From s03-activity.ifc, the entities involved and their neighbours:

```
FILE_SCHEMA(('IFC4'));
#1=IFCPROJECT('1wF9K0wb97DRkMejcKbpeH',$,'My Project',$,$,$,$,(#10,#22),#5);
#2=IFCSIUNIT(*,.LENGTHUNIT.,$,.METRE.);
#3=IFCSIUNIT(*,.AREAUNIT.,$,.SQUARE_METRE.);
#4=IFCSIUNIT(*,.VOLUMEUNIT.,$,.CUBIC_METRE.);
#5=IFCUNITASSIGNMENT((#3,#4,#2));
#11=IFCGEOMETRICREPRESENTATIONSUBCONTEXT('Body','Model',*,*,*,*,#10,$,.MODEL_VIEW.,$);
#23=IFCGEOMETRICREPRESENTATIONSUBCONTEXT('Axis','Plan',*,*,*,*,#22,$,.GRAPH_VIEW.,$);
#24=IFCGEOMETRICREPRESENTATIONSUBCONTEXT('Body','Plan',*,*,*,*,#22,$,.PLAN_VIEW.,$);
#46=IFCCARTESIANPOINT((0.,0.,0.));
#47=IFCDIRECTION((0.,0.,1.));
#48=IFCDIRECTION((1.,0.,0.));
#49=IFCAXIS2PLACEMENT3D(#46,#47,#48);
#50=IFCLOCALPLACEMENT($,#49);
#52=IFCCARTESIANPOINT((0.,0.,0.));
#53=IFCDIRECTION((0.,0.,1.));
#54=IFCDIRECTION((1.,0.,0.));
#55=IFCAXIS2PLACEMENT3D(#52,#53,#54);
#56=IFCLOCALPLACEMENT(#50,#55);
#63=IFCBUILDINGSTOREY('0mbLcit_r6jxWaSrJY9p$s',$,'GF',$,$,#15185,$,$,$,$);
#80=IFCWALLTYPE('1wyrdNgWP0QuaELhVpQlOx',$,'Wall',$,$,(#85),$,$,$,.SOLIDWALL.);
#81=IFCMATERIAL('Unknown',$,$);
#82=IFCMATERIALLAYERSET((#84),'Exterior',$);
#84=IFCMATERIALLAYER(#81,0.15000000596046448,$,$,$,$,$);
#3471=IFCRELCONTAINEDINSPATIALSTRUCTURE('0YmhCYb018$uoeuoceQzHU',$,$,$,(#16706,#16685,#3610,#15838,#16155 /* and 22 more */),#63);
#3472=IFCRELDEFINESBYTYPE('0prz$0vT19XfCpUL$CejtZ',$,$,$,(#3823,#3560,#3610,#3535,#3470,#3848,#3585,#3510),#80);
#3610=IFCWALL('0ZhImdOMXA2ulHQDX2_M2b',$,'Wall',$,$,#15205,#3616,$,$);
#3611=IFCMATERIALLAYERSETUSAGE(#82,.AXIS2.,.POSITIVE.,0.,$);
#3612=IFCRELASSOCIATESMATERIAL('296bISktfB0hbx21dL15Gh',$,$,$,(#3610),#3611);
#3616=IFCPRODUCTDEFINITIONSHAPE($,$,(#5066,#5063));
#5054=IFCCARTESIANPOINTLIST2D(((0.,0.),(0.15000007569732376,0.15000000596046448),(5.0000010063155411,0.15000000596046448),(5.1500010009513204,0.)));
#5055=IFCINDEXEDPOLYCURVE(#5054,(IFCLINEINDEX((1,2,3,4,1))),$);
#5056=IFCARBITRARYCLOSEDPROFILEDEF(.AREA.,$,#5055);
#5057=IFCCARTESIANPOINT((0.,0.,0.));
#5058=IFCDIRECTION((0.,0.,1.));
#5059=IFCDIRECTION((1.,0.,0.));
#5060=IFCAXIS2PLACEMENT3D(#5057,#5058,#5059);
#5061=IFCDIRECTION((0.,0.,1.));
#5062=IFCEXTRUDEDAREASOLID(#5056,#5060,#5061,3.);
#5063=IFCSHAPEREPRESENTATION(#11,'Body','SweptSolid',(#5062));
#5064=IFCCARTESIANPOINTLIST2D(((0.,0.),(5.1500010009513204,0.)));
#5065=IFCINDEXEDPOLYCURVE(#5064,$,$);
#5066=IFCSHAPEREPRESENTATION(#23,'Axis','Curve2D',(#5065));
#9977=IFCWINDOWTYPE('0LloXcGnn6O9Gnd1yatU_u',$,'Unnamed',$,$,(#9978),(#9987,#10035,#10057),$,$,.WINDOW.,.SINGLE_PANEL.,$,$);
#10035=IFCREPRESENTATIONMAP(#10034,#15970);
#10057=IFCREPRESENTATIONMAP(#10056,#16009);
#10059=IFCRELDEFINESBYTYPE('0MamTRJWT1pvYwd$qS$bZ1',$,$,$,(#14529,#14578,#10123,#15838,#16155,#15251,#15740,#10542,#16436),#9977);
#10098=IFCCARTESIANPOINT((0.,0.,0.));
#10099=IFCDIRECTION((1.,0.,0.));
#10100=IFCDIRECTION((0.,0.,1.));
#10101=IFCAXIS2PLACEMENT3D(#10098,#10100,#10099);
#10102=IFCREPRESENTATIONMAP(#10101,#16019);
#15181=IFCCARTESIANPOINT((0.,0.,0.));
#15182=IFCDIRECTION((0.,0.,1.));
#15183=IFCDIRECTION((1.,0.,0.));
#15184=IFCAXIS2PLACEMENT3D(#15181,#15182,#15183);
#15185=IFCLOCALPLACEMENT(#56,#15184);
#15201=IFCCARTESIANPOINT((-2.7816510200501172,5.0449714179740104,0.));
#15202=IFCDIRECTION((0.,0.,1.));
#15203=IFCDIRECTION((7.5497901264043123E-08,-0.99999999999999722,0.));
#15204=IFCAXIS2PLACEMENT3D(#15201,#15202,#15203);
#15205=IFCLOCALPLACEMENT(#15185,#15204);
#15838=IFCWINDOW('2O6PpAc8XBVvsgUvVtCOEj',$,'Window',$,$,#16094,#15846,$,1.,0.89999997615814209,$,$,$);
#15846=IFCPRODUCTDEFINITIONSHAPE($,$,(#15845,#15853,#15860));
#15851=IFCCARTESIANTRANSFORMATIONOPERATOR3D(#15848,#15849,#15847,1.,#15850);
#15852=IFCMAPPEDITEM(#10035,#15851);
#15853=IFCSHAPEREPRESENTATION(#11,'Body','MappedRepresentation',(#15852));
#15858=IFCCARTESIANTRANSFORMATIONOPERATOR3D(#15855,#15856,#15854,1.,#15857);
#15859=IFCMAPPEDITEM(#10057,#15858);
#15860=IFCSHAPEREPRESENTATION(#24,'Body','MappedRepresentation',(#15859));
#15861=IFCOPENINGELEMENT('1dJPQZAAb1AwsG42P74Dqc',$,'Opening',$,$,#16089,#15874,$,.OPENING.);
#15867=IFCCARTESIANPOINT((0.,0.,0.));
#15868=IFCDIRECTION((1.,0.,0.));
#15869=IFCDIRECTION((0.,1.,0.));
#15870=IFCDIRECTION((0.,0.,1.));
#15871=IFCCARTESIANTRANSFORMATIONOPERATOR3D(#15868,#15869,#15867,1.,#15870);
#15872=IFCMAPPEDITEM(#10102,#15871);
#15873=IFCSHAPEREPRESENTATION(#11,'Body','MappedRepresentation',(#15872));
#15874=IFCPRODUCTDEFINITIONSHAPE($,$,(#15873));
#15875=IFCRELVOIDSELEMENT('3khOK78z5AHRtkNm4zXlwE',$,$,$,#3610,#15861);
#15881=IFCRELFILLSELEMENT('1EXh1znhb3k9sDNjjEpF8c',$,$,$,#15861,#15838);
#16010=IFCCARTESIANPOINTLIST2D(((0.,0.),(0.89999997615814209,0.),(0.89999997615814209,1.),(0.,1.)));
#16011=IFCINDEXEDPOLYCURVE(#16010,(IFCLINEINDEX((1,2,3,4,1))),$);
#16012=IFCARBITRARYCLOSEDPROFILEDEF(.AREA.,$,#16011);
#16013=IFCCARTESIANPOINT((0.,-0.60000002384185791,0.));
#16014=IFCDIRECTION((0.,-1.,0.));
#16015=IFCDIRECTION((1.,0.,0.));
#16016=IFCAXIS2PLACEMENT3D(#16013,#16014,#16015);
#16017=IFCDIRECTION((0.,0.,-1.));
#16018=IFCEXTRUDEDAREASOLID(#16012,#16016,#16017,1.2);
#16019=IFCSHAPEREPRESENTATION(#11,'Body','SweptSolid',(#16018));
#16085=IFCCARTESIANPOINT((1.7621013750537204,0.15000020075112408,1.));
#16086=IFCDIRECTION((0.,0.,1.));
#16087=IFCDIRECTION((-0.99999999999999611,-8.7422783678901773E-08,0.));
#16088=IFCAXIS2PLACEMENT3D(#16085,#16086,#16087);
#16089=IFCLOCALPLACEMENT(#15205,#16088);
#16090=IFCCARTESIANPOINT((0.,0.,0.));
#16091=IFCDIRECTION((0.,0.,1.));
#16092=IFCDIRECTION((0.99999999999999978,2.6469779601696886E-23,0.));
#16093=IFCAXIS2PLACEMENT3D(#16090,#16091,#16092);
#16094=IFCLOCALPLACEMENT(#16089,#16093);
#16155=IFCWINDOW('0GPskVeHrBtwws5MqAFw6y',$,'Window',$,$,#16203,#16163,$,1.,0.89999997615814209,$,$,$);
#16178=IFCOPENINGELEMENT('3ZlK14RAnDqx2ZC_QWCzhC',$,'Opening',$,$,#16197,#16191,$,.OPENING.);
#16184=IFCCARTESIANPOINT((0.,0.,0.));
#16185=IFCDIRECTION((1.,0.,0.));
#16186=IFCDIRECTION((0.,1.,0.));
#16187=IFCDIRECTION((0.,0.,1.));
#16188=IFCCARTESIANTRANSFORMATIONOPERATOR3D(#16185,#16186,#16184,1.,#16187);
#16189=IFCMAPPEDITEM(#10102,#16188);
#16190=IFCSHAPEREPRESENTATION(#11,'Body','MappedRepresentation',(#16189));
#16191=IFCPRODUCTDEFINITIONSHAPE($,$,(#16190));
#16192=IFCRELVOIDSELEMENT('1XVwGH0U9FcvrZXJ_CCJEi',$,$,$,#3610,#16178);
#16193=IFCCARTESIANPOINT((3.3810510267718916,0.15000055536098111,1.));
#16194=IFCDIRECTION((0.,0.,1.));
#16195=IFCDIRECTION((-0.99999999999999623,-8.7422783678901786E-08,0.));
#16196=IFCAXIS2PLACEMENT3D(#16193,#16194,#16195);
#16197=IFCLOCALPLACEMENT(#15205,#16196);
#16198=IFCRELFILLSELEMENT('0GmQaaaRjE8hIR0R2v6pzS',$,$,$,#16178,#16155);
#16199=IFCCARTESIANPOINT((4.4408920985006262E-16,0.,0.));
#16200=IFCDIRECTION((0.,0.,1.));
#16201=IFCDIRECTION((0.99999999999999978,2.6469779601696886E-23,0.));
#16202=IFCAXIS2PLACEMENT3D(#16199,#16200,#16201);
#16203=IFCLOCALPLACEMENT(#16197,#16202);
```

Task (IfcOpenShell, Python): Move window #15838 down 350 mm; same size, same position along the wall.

```python
import numpy as np
import ifcopenshell
import ifcopenshell.api.geometry
import ifcopenshell.util.placement
import ifcopenshell.util.unit

model = ifcopenshell.open("s03-activity.ifc")
unit_scale = ifcopenshell.util.unit.calculate_unit_scale(model)

window = model.by_guid("2O6PpAc8XBVvsgUvVtCOEj")
opening = window.FillsVoids[0].RelatingOpeningElement
dz = -0.35 / unit_scale

shift = np.array([0.0, 0.0, dz])
# The window is placed relative to its opening, so it follows when the opening moves.
matrix = ifcopenshell.util.placement.get_local_placement(opening.ObjectPlacement)
matrix[:3, 3] += shift
ifcopenshell.api.geometry.edit_object_placement(
    model, product=opening, matrix=matrix, is_si=False, should_transform_children=True
)

print(f"moved by {dz * unit_scale:+.3f} m")

model.write("s03-activity_edited.ifc")
```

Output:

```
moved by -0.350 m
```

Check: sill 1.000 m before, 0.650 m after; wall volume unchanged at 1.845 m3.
